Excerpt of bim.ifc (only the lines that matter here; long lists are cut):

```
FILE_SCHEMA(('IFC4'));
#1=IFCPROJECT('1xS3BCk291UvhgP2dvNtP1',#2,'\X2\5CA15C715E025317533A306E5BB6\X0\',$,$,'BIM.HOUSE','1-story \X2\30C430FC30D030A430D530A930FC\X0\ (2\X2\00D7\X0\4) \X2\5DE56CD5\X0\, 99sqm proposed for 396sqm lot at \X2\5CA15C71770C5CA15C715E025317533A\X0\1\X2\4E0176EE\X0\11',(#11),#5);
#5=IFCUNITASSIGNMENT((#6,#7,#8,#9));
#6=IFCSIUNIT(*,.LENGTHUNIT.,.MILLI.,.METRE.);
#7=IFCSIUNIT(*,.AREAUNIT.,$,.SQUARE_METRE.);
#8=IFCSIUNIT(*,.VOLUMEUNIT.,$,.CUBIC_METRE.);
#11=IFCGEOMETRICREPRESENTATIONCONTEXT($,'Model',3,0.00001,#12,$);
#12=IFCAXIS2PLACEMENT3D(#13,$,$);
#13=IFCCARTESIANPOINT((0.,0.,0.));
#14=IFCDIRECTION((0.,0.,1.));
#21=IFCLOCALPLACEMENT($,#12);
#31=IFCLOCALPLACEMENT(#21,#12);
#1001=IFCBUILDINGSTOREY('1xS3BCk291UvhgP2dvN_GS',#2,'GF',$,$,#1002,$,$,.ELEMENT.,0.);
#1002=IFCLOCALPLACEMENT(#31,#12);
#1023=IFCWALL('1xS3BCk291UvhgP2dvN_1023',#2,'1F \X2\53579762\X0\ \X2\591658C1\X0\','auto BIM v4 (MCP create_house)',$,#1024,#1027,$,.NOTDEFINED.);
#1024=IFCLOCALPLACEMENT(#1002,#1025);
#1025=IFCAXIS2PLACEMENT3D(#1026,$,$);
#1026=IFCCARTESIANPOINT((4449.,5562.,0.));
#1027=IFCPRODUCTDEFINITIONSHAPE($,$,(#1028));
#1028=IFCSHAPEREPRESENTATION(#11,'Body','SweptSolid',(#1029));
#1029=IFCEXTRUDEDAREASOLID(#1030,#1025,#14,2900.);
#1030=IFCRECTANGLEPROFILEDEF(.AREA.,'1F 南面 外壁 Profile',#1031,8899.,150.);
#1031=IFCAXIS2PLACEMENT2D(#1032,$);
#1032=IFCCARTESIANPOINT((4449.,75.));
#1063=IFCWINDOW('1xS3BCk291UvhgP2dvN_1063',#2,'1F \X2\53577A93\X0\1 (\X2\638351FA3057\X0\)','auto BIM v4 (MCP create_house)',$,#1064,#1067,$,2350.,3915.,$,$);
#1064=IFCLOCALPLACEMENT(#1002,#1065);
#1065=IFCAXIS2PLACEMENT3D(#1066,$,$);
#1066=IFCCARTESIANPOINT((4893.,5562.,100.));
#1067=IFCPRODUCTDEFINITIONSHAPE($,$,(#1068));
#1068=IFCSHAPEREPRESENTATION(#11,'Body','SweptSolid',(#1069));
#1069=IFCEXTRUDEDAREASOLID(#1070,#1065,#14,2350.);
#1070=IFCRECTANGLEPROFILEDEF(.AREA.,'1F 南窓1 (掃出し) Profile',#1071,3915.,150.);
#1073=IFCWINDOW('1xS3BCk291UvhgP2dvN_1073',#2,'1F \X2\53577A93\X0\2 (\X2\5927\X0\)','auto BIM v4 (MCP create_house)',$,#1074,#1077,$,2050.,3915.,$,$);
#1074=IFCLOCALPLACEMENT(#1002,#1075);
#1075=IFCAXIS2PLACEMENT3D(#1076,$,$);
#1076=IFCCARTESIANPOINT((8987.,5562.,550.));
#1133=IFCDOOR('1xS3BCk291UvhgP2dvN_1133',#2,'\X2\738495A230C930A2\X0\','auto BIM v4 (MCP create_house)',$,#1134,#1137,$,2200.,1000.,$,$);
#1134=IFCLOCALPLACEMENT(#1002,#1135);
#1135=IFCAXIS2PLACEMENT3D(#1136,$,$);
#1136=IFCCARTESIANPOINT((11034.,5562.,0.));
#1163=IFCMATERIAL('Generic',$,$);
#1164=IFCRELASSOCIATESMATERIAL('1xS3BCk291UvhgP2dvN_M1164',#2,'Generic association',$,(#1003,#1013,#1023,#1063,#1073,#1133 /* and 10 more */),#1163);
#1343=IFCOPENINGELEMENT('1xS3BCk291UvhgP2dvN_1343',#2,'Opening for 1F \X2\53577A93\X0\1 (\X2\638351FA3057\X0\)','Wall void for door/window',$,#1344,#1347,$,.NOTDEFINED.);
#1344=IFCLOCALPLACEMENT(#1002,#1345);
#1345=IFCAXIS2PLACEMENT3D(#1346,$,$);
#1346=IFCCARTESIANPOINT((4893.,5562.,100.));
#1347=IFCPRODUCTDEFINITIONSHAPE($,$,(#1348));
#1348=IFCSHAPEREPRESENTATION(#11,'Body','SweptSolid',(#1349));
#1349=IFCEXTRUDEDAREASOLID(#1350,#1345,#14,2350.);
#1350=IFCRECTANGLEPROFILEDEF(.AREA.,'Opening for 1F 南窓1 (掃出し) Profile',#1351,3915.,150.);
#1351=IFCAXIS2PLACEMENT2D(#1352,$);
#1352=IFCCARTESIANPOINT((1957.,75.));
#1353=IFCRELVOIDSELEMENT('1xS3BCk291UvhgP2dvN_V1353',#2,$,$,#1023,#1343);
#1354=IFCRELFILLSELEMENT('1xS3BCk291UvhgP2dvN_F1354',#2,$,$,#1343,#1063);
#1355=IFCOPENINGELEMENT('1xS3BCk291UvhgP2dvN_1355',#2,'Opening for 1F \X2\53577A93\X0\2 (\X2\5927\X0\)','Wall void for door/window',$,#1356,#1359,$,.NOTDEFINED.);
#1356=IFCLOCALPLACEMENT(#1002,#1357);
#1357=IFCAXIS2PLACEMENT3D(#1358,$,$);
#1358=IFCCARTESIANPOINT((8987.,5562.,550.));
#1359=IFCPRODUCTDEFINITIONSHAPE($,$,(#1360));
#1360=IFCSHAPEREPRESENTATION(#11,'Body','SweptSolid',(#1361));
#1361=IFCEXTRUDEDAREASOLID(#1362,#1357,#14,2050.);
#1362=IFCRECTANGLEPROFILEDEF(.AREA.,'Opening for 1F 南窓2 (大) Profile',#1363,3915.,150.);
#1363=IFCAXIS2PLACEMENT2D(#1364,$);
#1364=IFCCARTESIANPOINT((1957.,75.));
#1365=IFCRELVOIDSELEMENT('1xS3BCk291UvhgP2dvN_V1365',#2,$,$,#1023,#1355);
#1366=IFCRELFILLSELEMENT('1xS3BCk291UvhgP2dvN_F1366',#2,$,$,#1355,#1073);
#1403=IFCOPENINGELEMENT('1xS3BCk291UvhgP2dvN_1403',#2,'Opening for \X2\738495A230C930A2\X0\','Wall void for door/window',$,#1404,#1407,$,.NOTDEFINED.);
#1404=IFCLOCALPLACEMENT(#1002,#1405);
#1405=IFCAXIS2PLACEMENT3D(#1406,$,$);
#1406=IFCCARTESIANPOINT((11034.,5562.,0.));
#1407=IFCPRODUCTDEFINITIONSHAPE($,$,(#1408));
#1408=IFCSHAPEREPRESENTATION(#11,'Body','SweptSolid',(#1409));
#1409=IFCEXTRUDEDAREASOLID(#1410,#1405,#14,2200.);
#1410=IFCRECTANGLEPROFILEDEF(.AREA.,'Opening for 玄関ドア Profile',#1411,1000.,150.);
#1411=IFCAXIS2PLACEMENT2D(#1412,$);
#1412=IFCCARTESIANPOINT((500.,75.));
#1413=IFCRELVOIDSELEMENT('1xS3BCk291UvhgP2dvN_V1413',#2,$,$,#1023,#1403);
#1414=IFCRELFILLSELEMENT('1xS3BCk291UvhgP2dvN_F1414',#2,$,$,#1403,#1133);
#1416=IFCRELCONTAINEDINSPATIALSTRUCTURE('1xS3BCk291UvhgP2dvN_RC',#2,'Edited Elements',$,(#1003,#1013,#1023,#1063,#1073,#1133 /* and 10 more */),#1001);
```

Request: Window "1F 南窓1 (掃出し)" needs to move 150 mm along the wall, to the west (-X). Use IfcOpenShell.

```python
import ifcopenshell
import ifcopenshell.api.geometry
import ifcopenshell.util.placement

model = ifcopenshell.open("bim.ifc")

window = model.by_guid("1xS3BCk291UvhgP2dvN_1063")
opening = window.FillsVoids[0].RelatingOpeningElement
wall = opening.VoidsElements[0].RelatingBuildingElement

wall_matrix = ifcopenshell.util.placement.get_local_placement(wall.ObjectPlacement)
shift = wall_matrix[:3, 0] * -150.0
before = ifcopenshell.util.placement.get_local_placement(window.ObjectPlacement)[:3, 3].copy()

# The window is not placed relative to its opening, so move both.
for product in (opening, window):
    matrix = ifcopenshell.util.placement.get_local_placement(product.ObjectPlacement)
    matrix[:3, 3] += shift
    ifcopenshell.api.geometry.edit_object_placement(model, product=product, matrix=matrix, is_si=False)

after = ifcopenshell.util.placement.get_local_placement(window.ObjectPlacement)[:3, 3]
print("window moved by", (after - before).round(3) + 0.0)

model.write("bim_v2.ifc")
```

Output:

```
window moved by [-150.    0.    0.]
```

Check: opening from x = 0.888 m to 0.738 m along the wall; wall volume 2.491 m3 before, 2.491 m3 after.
